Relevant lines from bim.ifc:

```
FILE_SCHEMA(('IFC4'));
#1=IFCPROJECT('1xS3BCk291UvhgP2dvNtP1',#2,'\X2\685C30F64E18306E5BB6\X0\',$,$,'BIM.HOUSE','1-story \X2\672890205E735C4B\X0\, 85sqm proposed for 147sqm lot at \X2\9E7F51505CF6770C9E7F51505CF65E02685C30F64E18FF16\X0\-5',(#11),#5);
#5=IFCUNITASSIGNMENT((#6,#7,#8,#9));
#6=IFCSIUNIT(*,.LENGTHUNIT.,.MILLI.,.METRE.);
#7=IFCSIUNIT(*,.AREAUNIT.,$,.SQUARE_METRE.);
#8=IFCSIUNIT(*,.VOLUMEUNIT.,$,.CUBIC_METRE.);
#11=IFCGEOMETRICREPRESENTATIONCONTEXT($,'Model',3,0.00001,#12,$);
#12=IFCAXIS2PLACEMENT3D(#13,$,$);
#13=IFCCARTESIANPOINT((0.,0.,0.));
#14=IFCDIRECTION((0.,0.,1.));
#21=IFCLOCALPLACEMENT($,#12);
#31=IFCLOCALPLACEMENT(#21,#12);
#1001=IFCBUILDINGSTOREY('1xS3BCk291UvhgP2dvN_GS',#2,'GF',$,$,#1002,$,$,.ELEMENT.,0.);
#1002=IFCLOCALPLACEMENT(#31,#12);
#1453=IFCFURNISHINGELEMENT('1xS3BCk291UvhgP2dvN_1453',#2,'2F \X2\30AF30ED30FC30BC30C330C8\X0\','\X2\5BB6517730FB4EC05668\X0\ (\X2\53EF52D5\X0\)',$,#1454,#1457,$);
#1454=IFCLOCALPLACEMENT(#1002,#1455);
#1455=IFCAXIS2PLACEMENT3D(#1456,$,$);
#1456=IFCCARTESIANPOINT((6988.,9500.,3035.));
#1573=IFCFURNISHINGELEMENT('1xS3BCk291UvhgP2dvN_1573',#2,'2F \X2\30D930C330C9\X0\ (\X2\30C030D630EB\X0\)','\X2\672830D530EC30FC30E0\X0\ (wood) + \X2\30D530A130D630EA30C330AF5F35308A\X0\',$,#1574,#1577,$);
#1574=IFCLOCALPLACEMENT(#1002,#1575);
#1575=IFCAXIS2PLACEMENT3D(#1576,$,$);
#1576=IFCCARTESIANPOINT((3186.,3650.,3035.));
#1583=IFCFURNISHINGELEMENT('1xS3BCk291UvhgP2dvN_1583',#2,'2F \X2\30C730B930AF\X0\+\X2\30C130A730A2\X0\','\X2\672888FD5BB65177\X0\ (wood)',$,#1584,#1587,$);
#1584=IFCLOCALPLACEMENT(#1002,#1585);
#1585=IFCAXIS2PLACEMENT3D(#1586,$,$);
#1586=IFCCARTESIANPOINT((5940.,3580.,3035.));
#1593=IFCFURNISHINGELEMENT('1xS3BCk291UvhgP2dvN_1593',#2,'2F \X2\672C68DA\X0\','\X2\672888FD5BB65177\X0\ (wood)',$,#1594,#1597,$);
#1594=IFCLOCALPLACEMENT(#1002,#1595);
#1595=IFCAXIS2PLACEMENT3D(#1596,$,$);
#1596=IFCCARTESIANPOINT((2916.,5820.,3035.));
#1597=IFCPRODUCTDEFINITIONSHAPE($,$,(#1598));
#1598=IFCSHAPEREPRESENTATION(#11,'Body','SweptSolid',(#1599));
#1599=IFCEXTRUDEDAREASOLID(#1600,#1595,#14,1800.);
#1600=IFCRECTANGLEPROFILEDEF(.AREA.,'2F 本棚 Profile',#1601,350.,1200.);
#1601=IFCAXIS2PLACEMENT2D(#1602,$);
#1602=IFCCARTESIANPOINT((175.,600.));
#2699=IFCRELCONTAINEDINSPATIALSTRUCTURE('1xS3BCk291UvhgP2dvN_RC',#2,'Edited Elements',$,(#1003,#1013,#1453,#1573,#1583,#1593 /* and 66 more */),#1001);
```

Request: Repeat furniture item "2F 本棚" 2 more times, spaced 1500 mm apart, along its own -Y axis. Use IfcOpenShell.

```python
import ifcopenshell
import ifcopenshell.api.geometry
import ifcopenshell.api.root
import ifcopenshell.util.element
import ifcopenshell.util.placement
import ifcopenshell.util.unit

model = ifcopenshell.open("bim.ifc")
unit_scale = ifcopenshell.util.unit.calculate_unit_scale(model)


def reuse_history(source, copy):
    """copy_class also copies each property set's owner history, people and application; keep the originals."""
    for rel in copy.IsDefinedBy:
        if rel.is_a("IfcRelDefinesByProperties") and (history := rel.RelatingPropertyDefinition.OwnerHistory):
            rel.RelatingPropertyDefinition.OwnerHistory = source.OwnerHistory
            ifcopenshell.util.element.remove_deep2(model, history)


source = model.by_guid("1xS3BCk291UvhgP2dvN_1593")
base = ifcopenshell.util.placement.get_local_placement(source.ObjectPlacement)
step = -base[:3, 1] * 1.5 / unit_scale

for i in range(1, 3):
    copy = ifcopenshell.api.root.copy_class(model, product=source)
    copy.Representation = ifcopenshell.util.element.copy_deep(
        model, source.Representation, exclude=["IfcGeometricRepresentationContext", "IfcRepresentationMap"]
    )
    reuse_history(source, copy)
    matrix = base.copy()
    matrix[:3, 3] += i * step
    print("added at", matrix[:3, 3].round(3) + 0.0)
    ifcopenshell.api.geometry.edit_object_placement(model, product=copy, matrix=matrix, is_si=False)

model.write("bim_updated.ifc")
```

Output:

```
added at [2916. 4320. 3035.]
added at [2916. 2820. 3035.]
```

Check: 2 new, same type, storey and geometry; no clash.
